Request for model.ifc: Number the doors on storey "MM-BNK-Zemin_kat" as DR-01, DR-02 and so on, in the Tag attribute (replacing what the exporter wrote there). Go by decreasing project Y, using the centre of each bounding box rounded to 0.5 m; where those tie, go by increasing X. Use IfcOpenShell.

First a look at what the model holds.

```python
import ifcopenshell
import ifcopenshell.util.element
import ifcopenshell.util.placement

model = ifcopenshell.open("model.ifc")
print(model.schema)
storey = next(s for s in model.by_type("IfcBuildingStorey") if s.Name == "MM-BNK-Zemin_kat")
doors = [e for e in ifcopenshell.util.element.get_decomposition(storey) if e.is_a("IfcDoor")]
for e in sorted(doors, key=lambda e: e.id()):
    origin = ifcopenshell.util.placement.get_local_placement(e.ObjectPlacement)[:3, 3]
    print(e.id(), e.Tag, e.Name, origin.round(2) + 0.0, sep=" | ")
```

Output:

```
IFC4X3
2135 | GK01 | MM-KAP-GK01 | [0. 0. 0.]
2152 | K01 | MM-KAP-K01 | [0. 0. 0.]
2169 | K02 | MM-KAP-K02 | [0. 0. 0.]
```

```python
import ifcopenshell
import ifcopenshell.geom
import ifcopenshell.util.element
import ifcopenshell.util.shape

model = ifcopenshell.open("model.ifc")
settings = ifcopenshell.geom.settings()
settings.set("use-world-coords", True)


def centre(element):
    shape = ifcopenshell.geom.create_shape(settings, element)
    return ifcopenshell.util.shape.get_bbox_centroid(shape.geometry)


storey = next(s for s in model.by_type("IfcBuildingStorey") if s.Name == "MM-BNK-Zemin_kat")
doors = [e for e in ifcopenshell.util.element.get_decomposition(storey) if e.is_a("IfcDoor")]

# Insertion points can sit at a corner or the storey origin, so sort by the geometry (in metres).
centres = {e: centre(e) for e in doors}
doors.sort(key=lambda e: (-round(centres[e][1] / 0.5), centres[e][0]))

for i, e in enumerate(doors, start=1):
    number = f"DR-{i:02d}"
    e.Tag = number
    print(e.id(), number)

model.write("model-out.ifc")
```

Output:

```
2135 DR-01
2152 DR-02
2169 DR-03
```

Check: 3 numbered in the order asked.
